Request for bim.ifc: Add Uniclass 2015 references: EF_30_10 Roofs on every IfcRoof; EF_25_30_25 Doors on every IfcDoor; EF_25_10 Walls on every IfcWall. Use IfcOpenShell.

First a look at what the model holds.

```python
import ifcopenshell

model = ifcopenshell.open("bim.ifc")
print(model.schema)
print("classifications:", [c.Name for c in model.by_type("IfcClassification")])
for ifc_class in ("IfcDoor", "IfcRoof", "IfcStair", "IfcWall", "IfcWindow"):
    print(ifc_class, len(model.by_type(ifc_class)))
```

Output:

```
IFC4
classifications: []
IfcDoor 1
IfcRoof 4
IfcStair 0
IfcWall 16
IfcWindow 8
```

```python
import ifcopenshell
import ifcopenshell.api.classification

model = ifcopenshell.open("bim.ifc")

system = ifcopenshell.api.classification.add_classification(model, classification="Uniclass 2015")

codes = {
    "IfcRoof": ("EF_30_10", "Roofs"),
    "IfcDoor": ("EF_25_30_25", "Doors"),
    "IfcWall": ("EF_25_10", "Walls"),
}
for ifc_class, (code, name) in codes.items():
    products = model.by_type(ifc_class)
    ifcopenshell.api.classification.add_reference(
        model, products=products, classification=system, identification=code, name=name
    )
    print(code, len(products))

model.write("bim_edited.ifc")
```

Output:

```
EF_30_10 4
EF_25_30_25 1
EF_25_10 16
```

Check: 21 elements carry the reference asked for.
